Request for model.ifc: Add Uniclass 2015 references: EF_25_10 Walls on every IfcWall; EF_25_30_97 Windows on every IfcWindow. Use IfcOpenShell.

First a look at what the model holds.

```python
import ifcopenshell

model = ifcopenshell.open("model.ifc")
print(model.schema)
print("classifications:", [c.Name for c in model.by_type("IfcClassification")])
for ifc_class in ("IfcDoor", "IfcRoof", "IfcStair", "IfcWall", "IfcWindow"):
    print(ifc_class, len(model.by_type(ifc_class)))
```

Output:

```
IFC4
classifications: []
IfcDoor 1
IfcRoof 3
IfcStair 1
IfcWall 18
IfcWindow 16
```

```python
import ifcopenshell
import ifcopenshell.api.classification

model = ifcopenshell.open("model.ifc")

system = ifcopenshell.api.classification.add_classification(model, classification="Uniclass 2015")

codes = {
    "IfcWall": ("EF_25_10", "Walls"),
    "IfcWindow": ("EF_25_30_97", "Windows"),
}
for ifc_class, (code, name) in codes.items():
    products = model.by_type(ifc_class)
    ifcopenshell.api.classification.add_reference(
        model, products=products, classification=system, identification=code, name=name
    )
    print(code, len(products))

model.write("model_v2.ifc")
```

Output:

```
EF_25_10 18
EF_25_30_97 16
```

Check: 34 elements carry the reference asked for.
